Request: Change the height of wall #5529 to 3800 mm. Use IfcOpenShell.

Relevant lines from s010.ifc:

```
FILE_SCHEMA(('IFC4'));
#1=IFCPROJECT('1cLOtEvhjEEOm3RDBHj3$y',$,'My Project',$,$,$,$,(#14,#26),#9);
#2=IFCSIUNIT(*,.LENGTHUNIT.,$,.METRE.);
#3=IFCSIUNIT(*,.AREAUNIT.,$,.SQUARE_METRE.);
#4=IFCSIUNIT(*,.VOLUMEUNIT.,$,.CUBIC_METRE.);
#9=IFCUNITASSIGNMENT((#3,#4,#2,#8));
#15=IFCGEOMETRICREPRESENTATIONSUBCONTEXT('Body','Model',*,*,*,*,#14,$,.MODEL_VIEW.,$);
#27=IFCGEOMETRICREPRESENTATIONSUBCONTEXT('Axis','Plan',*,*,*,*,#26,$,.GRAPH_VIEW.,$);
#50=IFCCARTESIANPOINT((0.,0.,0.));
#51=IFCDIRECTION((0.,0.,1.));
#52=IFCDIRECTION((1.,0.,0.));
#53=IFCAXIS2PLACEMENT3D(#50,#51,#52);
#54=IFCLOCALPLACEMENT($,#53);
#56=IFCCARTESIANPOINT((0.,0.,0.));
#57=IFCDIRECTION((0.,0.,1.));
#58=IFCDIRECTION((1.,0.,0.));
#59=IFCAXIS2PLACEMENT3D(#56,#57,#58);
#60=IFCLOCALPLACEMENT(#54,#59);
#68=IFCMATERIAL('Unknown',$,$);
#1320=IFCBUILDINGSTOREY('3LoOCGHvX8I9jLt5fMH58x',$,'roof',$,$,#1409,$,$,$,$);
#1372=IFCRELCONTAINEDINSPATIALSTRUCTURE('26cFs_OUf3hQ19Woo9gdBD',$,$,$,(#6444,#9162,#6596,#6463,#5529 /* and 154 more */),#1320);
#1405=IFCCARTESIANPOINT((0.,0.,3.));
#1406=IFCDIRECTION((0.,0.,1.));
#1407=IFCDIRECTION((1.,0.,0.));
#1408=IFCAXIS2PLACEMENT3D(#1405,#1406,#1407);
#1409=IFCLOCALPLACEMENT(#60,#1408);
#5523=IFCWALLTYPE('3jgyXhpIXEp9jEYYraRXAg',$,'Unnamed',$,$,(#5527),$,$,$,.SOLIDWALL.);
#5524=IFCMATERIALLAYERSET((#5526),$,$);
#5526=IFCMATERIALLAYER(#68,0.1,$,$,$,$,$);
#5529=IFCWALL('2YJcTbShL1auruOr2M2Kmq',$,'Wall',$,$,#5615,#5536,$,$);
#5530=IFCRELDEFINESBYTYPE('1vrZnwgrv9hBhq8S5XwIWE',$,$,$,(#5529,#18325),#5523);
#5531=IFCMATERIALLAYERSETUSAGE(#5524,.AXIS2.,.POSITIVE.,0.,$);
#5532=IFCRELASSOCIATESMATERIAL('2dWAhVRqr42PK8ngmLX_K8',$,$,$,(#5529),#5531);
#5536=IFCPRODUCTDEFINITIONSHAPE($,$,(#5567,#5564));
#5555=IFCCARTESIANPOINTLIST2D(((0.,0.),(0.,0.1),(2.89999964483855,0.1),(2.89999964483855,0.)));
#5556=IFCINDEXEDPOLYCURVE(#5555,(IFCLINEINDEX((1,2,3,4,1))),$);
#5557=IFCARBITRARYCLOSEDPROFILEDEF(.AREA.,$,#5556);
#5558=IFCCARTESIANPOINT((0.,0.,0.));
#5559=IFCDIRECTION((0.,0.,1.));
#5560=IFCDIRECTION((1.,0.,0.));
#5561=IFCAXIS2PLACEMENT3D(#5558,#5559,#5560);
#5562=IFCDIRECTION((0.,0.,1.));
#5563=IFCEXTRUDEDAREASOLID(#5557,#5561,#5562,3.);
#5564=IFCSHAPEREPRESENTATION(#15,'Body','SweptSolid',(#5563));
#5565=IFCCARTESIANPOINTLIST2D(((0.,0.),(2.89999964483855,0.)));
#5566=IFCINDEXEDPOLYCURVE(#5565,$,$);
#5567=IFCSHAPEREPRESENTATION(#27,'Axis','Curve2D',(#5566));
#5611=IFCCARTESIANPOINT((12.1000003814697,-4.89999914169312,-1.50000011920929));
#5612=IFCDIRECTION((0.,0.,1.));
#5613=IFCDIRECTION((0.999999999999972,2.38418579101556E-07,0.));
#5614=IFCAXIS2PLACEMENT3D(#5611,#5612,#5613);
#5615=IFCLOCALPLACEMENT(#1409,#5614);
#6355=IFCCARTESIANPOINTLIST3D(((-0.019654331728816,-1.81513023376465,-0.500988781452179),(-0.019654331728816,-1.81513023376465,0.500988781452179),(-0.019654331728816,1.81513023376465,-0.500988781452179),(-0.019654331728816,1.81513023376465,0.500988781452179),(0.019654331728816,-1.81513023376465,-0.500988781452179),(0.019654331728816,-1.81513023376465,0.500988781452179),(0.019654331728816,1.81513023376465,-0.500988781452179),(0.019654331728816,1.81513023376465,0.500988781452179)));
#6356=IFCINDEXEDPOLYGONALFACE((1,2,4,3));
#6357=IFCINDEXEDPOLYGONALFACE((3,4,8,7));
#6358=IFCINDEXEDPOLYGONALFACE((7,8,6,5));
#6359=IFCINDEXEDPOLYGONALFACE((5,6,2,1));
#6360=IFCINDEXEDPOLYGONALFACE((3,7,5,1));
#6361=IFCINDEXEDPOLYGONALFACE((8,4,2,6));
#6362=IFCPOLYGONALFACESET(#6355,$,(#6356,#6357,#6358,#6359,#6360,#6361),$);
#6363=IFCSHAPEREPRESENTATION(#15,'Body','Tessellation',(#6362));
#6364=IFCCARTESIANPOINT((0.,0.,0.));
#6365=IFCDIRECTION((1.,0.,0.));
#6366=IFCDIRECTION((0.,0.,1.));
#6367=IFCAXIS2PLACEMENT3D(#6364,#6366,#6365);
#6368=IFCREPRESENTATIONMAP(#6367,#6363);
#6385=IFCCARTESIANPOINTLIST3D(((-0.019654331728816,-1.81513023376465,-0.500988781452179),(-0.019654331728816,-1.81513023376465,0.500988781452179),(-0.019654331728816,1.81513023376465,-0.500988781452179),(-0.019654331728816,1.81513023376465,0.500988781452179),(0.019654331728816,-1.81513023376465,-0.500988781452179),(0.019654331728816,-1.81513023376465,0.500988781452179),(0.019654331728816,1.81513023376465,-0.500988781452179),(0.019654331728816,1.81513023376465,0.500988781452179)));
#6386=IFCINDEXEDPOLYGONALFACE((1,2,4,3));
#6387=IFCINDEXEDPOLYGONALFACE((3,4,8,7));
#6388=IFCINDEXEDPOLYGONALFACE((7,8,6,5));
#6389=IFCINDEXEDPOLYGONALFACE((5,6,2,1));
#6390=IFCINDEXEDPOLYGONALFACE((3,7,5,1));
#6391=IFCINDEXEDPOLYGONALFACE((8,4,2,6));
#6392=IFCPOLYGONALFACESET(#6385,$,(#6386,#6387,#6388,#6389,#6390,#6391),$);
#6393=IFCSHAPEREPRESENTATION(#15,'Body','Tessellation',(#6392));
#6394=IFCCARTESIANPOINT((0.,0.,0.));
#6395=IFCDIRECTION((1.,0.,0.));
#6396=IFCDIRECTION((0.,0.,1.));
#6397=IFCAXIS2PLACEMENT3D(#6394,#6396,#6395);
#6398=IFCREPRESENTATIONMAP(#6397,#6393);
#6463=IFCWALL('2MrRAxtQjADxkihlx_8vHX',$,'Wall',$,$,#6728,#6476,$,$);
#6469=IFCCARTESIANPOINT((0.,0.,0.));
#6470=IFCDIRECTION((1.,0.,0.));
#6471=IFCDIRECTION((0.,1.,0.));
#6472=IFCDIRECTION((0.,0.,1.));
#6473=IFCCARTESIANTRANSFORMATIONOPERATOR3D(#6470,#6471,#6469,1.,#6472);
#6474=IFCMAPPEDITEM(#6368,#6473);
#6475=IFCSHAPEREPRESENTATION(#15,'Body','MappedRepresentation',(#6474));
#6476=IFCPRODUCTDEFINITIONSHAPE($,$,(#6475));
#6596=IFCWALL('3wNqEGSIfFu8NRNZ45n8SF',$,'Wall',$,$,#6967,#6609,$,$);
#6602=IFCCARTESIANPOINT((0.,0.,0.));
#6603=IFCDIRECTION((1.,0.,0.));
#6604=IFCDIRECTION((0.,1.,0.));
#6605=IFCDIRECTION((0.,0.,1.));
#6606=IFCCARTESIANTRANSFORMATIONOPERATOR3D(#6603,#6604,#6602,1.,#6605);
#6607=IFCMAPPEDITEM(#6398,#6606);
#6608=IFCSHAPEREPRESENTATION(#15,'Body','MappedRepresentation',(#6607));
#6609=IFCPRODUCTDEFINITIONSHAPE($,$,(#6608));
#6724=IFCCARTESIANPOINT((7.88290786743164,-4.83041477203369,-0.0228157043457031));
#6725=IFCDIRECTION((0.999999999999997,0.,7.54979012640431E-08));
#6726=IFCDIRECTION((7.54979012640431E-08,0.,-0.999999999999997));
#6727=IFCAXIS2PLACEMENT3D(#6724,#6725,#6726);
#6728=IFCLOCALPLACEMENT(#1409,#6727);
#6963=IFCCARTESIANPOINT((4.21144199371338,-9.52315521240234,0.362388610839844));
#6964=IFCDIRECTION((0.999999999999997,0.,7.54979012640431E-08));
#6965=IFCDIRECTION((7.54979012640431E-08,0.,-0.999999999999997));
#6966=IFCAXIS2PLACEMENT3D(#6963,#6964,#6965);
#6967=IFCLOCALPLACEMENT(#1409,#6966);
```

```python
import ifcopenshell
import ifcopenshell.geom
import ifcopenshell.util.representation
import ifcopenshell.util.shape

model = ifcopenshell.open("s010.ifc")
settings = ifcopenshell.geom.settings()


def volume(element):
    """Net volume in cubic metres, openings subtracted."""
    shape = ifcopenshell.geom.create_shape(settings, element)
    return ifcopenshell.util.shape.get_volume(shape.geometry)


wall = model.by_guid("2YJcTbShL1auruOr2M2Kmq")
before = volume(wall)

body = ifcopenshell.util.representation.get_representation(wall, "Model", "Body")
solid = body.Items[0]
old_height = solid.Depth
solid.Depth = 3.8
after = volume(wall)

print(f"height {old_height:g} -> {solid.Depth:g}, volume {before:.3f} -> {after:.3f} m3")

model.write("s010_rev.ifc")
```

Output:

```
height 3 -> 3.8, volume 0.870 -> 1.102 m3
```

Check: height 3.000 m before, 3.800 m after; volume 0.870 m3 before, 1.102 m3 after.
